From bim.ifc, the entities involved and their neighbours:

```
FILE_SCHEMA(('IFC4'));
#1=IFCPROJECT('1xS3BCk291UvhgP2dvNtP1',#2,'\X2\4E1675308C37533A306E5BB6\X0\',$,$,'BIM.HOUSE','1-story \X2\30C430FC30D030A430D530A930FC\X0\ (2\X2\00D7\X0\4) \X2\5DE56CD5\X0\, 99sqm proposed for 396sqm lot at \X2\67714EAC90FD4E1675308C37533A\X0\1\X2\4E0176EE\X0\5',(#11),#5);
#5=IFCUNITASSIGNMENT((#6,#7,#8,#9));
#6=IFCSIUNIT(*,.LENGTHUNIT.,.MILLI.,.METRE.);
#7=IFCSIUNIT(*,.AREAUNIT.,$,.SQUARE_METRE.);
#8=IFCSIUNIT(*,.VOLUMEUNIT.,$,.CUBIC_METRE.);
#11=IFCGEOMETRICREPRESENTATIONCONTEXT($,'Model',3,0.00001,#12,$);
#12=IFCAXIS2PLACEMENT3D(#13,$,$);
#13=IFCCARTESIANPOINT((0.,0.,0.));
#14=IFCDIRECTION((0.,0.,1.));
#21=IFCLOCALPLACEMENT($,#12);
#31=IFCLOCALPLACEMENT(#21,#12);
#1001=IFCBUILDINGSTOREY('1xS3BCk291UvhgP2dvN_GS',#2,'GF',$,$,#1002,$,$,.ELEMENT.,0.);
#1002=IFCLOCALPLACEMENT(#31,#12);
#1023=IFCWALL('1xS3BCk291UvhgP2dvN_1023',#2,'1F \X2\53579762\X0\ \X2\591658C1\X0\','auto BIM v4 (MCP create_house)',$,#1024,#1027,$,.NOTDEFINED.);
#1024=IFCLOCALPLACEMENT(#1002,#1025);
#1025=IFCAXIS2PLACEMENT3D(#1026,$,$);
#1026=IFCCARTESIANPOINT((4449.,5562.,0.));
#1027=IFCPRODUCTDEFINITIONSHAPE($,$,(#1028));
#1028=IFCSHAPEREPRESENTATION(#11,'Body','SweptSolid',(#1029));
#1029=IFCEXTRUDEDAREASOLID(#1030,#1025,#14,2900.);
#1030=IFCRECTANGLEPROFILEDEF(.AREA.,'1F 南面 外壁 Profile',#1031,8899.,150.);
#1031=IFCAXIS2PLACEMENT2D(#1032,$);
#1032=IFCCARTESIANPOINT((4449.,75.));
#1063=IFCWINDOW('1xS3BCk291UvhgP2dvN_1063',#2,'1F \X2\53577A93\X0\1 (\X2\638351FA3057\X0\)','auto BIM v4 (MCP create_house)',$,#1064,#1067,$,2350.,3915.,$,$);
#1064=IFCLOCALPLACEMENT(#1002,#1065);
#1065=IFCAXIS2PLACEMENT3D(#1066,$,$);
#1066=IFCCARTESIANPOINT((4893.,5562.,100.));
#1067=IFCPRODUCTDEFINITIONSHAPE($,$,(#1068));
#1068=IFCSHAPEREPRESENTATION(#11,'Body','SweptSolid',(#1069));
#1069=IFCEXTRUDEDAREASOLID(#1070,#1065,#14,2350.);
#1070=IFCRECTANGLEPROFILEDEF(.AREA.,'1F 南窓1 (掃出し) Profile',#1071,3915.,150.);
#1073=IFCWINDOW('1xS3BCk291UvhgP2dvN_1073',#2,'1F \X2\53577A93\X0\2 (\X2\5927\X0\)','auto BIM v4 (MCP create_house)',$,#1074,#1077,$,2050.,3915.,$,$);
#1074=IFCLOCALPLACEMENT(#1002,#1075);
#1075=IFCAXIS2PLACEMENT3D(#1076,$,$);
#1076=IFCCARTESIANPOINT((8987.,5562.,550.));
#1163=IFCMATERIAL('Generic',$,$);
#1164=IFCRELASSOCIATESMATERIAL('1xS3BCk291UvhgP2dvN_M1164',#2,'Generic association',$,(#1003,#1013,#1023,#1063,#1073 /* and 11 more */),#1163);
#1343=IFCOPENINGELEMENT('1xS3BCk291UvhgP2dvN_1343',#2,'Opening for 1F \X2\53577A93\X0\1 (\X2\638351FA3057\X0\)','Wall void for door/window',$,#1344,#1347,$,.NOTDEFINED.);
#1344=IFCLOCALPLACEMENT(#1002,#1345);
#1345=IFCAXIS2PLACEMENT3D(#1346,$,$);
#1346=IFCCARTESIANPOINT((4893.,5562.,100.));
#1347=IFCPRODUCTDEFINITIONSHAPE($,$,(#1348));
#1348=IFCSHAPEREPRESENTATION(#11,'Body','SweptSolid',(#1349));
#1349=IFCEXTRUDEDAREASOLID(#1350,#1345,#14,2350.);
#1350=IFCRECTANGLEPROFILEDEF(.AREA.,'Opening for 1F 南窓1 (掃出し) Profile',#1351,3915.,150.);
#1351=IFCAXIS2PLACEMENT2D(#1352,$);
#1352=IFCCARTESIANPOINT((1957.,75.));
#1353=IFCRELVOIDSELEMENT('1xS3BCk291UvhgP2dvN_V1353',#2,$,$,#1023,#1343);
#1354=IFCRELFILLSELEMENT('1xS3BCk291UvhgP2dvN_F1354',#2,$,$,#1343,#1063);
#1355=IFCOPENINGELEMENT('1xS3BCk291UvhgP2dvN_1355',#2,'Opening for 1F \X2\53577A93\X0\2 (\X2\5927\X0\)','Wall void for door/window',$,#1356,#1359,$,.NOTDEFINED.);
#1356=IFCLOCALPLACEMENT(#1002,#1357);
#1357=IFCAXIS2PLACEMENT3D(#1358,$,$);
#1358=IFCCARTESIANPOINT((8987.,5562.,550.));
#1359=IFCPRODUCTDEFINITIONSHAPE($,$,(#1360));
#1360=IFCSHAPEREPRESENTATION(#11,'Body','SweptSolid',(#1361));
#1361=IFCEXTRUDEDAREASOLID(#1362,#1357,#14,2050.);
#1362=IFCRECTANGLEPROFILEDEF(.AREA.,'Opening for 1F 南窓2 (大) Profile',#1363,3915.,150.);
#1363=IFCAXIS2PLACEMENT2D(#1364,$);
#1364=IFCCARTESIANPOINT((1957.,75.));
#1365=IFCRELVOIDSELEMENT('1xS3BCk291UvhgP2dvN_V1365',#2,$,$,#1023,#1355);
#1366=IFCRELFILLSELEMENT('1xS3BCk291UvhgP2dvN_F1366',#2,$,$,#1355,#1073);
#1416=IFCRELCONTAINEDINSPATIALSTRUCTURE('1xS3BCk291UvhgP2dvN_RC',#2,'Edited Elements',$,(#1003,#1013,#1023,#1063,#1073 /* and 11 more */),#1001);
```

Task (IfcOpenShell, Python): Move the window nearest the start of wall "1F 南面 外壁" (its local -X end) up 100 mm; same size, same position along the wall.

```python
import numpy as np
import ifcopenshell
import ifcopenshell.api.geometry
import ifcopenshell.util.placement
import ifcopenshell.util.unit

model = ifcopenshell.open("bim.ifc")
unit_scale = ifcopenshell.util.unit.calculate_unit_scale(model)

window = model.by_guid("1xS3BCk291UvhgP2dvN_1063")
opening = window.FillsVoids[0].RelatingOpeningElement
dz = 0.1 / unit_scale

shift = np.array([0.0, 0.0, dz])
# The window is not placed relative to its opening, so move both.
for product in (opening, window):
    matrix = ifcopenshell.util.placement.get_local_placement(product.ObjectPlacement)
    matrix[:3, 3] += shift
    ifcopenshell.api.geometry.edit_object_placement(model, product=product, matrix=matrix, is_si=False)

print(f"moved by {dz * unit_scale:+.3f} m")

model.write("bim_rev.ifc")
```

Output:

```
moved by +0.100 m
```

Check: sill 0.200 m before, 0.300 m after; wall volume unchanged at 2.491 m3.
